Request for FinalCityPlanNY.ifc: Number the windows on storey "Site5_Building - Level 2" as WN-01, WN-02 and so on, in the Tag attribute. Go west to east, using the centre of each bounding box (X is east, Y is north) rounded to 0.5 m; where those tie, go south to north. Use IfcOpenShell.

First a look at what the model holds.

```python
import ifcopenshell
import ifcopenshell.util.element
import ifcopenshell.util.placement

model = ifcopenshell.open("FinalCityPlanNY.ifc")
print(model.schema)
storey = next(s for s in model.by_type("IfcBuildingStorey") if s.Name == "Site5_Building - Level 2")
windows = [e for e in ifcopenshell.util.element.get_decomposition(storey) if e.is_a("IfcWindow")]
for e in sorted(windows, key=lambda e: e.id()):
    origin = ifcopenshell.util.placement.get_local_placement(e.ObjectPlacement)[:3, 3]
    print(e.id(), e.Tag, e.Name, origin.round(2) + 0.0, sep=" | ")
```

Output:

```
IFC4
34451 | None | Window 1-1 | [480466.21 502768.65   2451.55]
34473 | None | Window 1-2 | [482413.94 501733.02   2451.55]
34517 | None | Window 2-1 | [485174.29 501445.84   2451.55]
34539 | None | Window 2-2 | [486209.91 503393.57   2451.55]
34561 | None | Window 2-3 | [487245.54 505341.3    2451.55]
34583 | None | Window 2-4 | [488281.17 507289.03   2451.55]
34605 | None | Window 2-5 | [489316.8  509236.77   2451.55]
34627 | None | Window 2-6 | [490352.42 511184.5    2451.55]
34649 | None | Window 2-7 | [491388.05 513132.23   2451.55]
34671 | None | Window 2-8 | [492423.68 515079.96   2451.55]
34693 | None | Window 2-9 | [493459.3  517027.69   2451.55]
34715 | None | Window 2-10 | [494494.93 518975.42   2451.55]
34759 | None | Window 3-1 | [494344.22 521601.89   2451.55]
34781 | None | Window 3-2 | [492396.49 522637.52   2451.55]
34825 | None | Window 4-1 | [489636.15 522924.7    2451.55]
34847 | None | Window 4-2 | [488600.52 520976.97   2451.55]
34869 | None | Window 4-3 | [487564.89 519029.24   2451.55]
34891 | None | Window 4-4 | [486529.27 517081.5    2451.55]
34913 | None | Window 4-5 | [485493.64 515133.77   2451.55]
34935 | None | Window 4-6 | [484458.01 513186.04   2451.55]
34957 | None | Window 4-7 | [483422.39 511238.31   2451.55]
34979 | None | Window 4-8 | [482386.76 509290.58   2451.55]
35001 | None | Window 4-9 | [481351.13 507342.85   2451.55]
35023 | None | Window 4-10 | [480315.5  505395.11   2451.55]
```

```python
import ifcopenshell
import ifcopenshell.geom
import ifcopenshell.util.element
import ifcopenshell.util.shape

model = ifcopenshell.open("FinalCityPlanNY.ifc")
settings = ifcopenshell.geom.settings()
settings.set("use-world-coords", True)


def centre(element):
    shape = ifcopenshell.geom.create_shape(settings, element)
    return ifcopenshell.util.shape.get_bbox_centroid(shape.geometry)


storey = next(s for s in model.by_type("IfcBuildingStorey") if s.Name == "Site5_Building - Level 2")
windows = [e for e in ifcopenshell.util.element.get_decomposition(storey) if e.is_a("IfcWindow")]

# Insertion points can sit at a corner or the storey origin, so sort by the geometry (in metres).
centres = {e: centre(e) for e in windows}
windows.sort(key=lambda e: (round(centres[e][0] / 0.5), centres[e][1]))

for i, e in enumerate(windows, start=1):
    number = f"WN-{i:02d}"
    e.Tag = number
    print(e.id(), number)

model.write("FinalCityPlanNY_v2.ifc")
```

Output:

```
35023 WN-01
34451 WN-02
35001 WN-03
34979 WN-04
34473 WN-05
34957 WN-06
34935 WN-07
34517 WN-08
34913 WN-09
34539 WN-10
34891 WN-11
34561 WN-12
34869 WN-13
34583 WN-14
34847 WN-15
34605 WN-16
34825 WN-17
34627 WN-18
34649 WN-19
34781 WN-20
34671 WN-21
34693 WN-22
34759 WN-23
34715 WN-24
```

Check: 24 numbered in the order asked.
